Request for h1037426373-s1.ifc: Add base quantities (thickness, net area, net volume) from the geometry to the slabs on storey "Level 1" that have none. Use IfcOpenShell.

First a look at what the model holds.

```python
import ifcopenshell
import ifcopenshell.util.element
import ifcopenshell.util.unit

model = ifcopenshell.open("h1037426373-s1.ifc")
print(model.schema)
for unit_type in ("LENGTHUNIT", "AREAUNIT", "VOLUMEUNIT"):
    print(unit_type, ifcopenshell.util.unit.calculate_unit_scale(model, unit_type))
storey = next(s for s in model.by_type("IfcBuildingStorey") if s.Name == "Level 1")
slabs = [e for e in ifcopenshell.util.element.get_decomposition(storey) if e.is_a("IfcSlab")]
for e in sorted(slabs, key=lambda e: e.id()):
    print(e.id(), e.is_a(), e.Name, list(ifcopenshell.util.element.get_psets(e, qtos_only=True)), sep=" | ")
```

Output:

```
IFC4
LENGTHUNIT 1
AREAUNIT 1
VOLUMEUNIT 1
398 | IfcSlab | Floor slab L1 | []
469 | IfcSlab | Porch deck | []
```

```python
import ifcopenshell
import ifcopenshell.api.pset
import ifcopenshell.geom
import ifcopenshell.util.element
import ifcopenshell.util.shape
import ifcopenshell.util.unit

model = ifcopenshell.open("h1037426373-s1.ifc")
unit_scale = ifcopenshell.util.unit.calculate_unit_scale(model)
area_scale = ifcopenshell.util.unit.calculate_unit_scale(model, "AREAUNIT")
volume_scale = ifcopenshell.util.unit.calculate_unit_scale(model, "VOLUMEUNIT")
settings = ifcopenshell.geom.settings()

storey = next(s for s in model.by_type("IfcBuildingStorey") if s.Name == "Level 1")
slabs = [e for e in ifcopenshell.util.element.get_decomposition(storey) if e.is_a("IfcSlab")]

for e in sorted(slabs, key=lambda e: e.id()):
    if ifcopenshell.util.element.get_psets(e, qtos_only=True, should_inherit=False):
        continue
    # Geometry comes back in metres, in the element's own axes.
    shape = ifcopenshell.geom.create_shape(settings, e)
    values = {
        "Width": ifcopenshell.util.shape.get_z(shape.geometry) / unit_scale,
        "NetArea": ifcopenshell.util.shape.get_footprint_area(shape.geometry) / area_scale,
        "NetVolume": ifcopenshell.util.shape.get_volume(shape.geometry) / volume_scale,
    }
    qto = ifcopenshell.api.pset.add_qto(model, product=e, name="Qto_SlabBaseQuantities")
    ifcopenshell.api.pset.edit_qto(model, qto=qto, properties=values)
    print(e.id(), {k: round(v, 3) for k, v in values.items()})

model.write("h1037426373-s1-out.ifc")
```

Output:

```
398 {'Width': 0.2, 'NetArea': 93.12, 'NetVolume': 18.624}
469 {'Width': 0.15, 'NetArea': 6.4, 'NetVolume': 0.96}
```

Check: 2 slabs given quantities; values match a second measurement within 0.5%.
